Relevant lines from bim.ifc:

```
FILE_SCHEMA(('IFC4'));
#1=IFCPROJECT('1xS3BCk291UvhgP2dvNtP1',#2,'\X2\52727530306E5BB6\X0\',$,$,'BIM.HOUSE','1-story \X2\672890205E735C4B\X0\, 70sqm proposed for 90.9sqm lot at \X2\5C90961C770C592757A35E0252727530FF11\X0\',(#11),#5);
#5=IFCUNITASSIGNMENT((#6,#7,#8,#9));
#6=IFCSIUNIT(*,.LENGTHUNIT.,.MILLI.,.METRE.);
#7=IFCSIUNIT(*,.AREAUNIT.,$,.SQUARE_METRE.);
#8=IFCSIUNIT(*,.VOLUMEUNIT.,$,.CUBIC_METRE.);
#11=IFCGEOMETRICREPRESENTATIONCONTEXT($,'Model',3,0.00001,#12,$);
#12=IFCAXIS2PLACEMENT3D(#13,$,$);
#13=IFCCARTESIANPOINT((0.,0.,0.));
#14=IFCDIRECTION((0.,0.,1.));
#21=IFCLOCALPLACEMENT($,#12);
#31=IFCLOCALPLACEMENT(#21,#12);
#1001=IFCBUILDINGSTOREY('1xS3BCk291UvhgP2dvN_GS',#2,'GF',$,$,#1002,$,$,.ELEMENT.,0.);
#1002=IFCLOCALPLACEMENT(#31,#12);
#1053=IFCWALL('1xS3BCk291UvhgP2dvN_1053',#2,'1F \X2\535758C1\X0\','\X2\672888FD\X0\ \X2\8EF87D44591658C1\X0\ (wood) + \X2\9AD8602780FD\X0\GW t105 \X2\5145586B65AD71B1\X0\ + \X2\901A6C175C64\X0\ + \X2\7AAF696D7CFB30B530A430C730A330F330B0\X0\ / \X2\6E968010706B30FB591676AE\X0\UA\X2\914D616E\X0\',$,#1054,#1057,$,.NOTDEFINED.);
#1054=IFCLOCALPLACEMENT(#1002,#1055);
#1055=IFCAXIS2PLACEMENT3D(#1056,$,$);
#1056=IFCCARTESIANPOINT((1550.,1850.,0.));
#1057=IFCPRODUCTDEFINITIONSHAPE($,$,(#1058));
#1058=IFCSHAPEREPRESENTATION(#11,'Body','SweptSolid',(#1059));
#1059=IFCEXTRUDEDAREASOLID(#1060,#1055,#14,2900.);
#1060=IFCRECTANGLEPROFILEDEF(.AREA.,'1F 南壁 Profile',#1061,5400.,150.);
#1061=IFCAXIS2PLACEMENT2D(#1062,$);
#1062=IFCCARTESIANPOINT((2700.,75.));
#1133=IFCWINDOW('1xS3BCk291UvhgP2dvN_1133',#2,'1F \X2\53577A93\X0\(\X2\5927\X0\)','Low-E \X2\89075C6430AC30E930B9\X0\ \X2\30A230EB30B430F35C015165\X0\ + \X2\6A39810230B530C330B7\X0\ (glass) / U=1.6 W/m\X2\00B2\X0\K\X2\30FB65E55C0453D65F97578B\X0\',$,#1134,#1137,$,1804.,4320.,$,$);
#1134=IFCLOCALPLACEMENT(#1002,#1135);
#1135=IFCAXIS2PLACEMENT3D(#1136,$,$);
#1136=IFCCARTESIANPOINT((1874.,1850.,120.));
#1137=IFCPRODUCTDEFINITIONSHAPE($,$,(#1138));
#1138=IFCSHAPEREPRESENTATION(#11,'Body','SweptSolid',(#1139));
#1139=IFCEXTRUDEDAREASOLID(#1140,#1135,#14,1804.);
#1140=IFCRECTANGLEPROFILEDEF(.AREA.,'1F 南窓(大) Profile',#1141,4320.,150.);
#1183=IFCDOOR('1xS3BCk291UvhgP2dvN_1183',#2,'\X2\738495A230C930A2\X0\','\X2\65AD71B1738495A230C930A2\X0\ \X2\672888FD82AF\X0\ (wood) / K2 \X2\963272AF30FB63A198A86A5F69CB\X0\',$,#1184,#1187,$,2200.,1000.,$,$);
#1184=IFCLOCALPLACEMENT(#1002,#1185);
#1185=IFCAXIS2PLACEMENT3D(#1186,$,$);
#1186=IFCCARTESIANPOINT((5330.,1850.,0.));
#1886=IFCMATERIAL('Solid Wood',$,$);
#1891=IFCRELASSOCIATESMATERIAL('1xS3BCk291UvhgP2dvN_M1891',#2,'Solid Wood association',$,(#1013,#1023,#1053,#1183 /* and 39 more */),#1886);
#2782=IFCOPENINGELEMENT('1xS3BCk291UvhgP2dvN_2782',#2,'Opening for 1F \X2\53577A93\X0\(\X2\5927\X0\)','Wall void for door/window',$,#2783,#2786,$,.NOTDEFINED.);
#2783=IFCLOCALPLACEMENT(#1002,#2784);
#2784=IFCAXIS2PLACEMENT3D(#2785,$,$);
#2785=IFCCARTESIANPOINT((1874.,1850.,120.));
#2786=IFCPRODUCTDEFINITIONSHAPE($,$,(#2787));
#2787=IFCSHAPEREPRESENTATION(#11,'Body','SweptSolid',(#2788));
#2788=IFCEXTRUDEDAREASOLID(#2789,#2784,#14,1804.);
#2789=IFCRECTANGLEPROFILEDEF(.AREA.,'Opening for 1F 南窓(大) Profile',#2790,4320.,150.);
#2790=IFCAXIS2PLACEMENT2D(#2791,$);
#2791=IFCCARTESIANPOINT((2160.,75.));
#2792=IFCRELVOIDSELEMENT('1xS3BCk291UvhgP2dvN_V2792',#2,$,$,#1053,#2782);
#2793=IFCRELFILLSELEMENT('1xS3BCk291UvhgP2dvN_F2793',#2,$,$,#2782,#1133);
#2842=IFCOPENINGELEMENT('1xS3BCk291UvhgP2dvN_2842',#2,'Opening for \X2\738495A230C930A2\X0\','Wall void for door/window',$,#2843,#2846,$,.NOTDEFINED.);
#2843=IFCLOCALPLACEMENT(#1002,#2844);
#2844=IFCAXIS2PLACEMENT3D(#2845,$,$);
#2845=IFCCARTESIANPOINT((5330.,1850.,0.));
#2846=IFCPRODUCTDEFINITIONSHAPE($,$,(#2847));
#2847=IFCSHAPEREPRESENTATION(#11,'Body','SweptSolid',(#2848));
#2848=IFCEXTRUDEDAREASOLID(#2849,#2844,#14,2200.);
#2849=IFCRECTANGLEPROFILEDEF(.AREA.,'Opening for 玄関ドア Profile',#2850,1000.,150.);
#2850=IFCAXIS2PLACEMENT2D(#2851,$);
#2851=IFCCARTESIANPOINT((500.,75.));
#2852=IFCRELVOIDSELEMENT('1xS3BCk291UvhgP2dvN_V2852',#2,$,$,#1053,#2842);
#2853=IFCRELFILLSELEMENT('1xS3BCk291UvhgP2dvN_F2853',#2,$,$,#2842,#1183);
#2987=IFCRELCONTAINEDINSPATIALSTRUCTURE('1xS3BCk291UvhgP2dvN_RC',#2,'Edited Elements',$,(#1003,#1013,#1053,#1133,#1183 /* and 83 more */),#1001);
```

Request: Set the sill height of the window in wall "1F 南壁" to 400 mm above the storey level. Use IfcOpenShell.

```python
import numpy as np
import ifcopenshell
import ifcopenshell.api.geometry
import ifcopenshell.geom
import ifcopenshell.util.element
import ifcopenshell.util.placement
import ifcopenshell.util.shape
import ifcopenshell.util.unit

model = ifcopenshell.open("bim.ifc")
unit_scale = ifcopenshell.util.unit.calculate_unit_scale(model)

window = model.by_id(1133)
opening = window.FillsVoids[0].RelatingOpeningElement
storey = ifcopenshell.util.element.get_container(window, ifc_class="IfcBuildingStorey")
level = ifcopenshell.util.placement.get_local_placement(storey.ObjectPlacement)[2, 3]

# The opening's origin need not be at the sill, so measure its lowest point.
shape = ifcopenshell.geom.create_shape(ifcopenshell.geom.settings(), opening)
bottom = ifcopenshell.util.shape.get_shape_bottom_elevation(shape, shape.geometry) / unit_scale
dz = level + 0.4 / unit_scale - bottom

shift = np.array([0.0, 0.0, dz])
# The window is not placed relative to its opening, so move both.
for product in (opening, window):
    matrix = ifcopenshell.util.placement.get_local_placement(product.ObjectPlacement)
    matrix[:3, 3] += shift
    ifcopenshell.api.geometry.edit_object_placement(model, product=product, matrix=matrix, is_si=False)

print(f"moved by {dz * unit_scale:+.3f} m")

model.write("bim_rev.ifc")
```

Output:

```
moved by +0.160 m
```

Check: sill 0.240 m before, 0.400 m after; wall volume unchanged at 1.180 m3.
